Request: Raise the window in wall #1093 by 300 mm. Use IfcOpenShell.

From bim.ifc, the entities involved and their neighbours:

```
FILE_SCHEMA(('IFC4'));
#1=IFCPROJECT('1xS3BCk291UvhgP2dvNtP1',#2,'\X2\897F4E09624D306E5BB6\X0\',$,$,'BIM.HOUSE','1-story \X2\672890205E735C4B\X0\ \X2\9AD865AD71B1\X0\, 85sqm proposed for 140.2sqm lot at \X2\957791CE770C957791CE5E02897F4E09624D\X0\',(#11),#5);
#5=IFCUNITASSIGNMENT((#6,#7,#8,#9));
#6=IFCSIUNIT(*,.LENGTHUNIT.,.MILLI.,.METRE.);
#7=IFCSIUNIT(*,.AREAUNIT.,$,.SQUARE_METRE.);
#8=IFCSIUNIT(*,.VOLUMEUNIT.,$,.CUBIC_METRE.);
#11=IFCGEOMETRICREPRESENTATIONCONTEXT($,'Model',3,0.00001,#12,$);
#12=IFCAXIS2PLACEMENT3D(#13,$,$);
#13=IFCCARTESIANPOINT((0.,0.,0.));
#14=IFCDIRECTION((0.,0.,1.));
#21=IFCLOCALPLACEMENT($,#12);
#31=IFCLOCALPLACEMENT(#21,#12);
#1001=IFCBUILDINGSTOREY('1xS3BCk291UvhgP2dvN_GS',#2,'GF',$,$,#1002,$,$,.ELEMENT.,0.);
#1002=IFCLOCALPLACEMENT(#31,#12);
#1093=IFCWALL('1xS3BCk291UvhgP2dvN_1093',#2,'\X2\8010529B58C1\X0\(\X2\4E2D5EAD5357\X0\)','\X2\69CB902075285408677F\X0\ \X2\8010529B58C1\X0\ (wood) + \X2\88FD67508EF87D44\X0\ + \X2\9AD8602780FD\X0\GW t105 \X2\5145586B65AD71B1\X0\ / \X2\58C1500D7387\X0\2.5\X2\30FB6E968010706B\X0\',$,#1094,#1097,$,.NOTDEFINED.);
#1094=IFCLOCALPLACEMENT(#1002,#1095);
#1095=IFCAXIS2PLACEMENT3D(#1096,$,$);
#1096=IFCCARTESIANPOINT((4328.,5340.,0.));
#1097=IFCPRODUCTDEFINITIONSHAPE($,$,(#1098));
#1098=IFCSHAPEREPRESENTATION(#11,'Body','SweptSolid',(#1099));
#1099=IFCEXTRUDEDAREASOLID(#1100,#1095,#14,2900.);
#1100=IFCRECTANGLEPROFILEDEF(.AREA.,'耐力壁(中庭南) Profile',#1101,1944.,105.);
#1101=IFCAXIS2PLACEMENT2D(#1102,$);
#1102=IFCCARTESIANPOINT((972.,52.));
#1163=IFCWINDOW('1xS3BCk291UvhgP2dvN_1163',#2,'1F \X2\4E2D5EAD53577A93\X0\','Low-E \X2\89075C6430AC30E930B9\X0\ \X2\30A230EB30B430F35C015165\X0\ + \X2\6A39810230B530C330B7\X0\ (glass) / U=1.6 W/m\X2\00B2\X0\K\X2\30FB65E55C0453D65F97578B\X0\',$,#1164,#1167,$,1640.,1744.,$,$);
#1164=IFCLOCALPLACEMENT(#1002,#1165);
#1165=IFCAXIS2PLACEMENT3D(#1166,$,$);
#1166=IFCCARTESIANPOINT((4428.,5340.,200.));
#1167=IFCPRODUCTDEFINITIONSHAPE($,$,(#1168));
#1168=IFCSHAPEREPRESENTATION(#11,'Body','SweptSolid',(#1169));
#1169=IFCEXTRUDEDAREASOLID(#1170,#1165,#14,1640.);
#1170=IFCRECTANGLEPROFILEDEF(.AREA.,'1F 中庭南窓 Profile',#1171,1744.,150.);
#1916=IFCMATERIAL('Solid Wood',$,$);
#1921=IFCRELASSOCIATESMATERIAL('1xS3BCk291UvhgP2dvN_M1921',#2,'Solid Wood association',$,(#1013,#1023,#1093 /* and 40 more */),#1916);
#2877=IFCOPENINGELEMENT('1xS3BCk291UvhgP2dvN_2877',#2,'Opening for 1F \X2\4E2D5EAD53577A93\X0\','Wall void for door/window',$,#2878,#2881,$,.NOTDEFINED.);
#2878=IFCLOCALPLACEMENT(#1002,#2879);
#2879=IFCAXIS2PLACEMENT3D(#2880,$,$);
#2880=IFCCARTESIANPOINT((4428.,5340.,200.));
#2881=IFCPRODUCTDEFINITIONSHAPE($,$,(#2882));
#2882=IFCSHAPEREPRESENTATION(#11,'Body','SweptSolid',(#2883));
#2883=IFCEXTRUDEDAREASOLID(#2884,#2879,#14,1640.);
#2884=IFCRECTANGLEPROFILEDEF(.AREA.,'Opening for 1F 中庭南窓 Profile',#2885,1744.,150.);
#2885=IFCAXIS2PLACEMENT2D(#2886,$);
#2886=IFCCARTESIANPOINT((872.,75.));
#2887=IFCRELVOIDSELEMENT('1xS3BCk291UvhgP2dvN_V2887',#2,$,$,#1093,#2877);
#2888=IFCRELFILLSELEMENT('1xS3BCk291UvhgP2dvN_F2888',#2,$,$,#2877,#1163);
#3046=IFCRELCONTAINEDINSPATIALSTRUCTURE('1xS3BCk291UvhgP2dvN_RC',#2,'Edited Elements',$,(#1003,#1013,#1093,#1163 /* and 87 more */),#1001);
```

```python
import numpy as np
import ifcopenshell
import ifcopenshell.api.geometry
import ifcopenshell.util.placement
import ifcopenshell.util.unit

model = ifcopenshell.open("bim.ifc")
unit_scale = ifcopenshell.util.unit.calculate_unit_scale(model)

window = model.by_guid("1xS3BCk291UvhgP2dvN_1163")
opening = window.FillsVoids[0].RelatingOpeningElement
dz = 0.3 / unit_scale

shift = np.array([0.0, 0.0, dz])
# The window is not placed relative to its opening, so move both.
for product in (opening, window):
    matrix = ifcopenshell.util.placement.get_local_placement(product.ObjectPlacement)
    matrix[:3, 3] += shift
    ifcopenshell.api.geometry.edit_object_placement(model, product=product, matrix=matrix, is_si=False)

print(f"moved by {dz * unit_scale:+.3f} m")

model.write("bim_v2.ifc")
```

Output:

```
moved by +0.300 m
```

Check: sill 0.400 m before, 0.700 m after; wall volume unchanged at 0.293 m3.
